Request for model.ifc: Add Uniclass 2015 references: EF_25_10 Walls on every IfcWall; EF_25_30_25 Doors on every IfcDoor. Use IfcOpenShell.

First a look at what the model holds.

```python
import ifcopenshell

model = ifcopenshell.open("model.ifc")
print(model.schema)
print("classifications:", [c.Name for c in model.by_type("IfcClassification")])
for ifc_class in ("IfcDoor", "IfcRoof", "IfcStair", "IfcWall", "IfcWindow"):
    print(ifc_class, len(model.by_type(ifc_class)))
```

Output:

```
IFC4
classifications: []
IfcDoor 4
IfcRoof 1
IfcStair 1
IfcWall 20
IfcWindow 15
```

```python
import ifcopenshell
import ifcopenshell.api.classification

model = ifcopenshell.open("model.ifc")

system = ifcopenshell.api.classification.add_classification(model, classification="Uniclass 2015")

codes = {
    "IfcWall": ("EF_25_10", "Walls"),
    "IfcDoor": ("EF_25_30_25", "Doors"),
}
for ifc_class, (code, name) in codes.items():
    products = model.by_type(ifc_class)
    ifcopenshell.api.classification.add_reference(
        model, products=products, classification=system, identification=code, name=name
    )
    print(code, len(products))

model.write("model-out.ifc")
```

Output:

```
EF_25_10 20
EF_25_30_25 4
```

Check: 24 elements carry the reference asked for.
